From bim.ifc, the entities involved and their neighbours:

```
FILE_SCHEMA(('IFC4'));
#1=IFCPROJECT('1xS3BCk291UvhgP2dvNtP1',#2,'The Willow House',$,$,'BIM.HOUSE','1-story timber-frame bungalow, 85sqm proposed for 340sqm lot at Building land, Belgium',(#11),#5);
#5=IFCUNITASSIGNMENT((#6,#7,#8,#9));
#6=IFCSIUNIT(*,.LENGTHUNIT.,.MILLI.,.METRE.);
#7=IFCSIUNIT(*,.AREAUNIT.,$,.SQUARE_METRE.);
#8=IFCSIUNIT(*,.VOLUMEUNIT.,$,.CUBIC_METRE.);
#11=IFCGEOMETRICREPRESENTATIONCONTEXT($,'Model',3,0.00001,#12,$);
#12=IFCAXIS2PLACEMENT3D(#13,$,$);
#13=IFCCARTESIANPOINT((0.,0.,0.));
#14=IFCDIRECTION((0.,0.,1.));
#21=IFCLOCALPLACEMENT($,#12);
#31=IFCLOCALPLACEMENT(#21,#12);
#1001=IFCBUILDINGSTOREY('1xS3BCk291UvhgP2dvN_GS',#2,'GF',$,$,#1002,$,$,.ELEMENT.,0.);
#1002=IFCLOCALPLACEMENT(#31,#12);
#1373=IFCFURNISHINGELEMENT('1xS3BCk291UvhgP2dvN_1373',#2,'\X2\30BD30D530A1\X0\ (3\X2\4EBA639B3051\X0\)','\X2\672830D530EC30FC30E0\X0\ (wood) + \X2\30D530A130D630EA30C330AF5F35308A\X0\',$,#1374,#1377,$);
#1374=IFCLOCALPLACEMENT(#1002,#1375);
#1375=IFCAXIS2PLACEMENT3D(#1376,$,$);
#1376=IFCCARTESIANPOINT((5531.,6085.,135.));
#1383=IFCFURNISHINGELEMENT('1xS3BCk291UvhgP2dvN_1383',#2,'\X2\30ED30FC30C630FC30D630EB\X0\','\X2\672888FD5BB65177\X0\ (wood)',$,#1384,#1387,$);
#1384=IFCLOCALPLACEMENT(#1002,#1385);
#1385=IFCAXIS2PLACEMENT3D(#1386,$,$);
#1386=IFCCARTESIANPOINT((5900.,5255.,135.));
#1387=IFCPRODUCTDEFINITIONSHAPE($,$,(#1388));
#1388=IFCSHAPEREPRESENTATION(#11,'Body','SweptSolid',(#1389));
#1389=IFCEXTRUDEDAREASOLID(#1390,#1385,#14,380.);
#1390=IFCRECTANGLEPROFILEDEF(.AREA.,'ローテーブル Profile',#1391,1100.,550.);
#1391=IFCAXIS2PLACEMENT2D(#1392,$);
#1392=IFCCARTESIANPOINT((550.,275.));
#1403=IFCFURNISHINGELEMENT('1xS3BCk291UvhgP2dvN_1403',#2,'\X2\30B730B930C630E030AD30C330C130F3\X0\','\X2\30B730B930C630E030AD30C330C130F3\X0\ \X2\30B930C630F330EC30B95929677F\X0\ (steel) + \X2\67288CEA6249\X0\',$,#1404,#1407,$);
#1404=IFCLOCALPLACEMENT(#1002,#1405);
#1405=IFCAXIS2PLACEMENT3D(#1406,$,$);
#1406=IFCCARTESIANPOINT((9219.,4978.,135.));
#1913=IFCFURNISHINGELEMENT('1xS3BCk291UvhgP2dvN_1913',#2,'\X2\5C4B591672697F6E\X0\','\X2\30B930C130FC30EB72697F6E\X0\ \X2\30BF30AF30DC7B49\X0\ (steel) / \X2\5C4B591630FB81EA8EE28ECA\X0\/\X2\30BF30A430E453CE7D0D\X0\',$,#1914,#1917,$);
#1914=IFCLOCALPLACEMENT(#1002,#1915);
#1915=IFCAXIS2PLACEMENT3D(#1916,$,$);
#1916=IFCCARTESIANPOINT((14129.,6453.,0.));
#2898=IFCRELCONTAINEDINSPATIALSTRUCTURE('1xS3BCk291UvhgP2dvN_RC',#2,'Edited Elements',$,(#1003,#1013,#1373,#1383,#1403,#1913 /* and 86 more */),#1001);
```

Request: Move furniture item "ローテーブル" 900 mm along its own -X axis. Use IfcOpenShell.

```python
import ifcopenshell
import ifcopenshell.api.geometry
import ifcopenshell.util.placement

model = ifcopenshell.open("bim.ifc")

item = model.by_guid("1xS3BCk291UvhgP2dvN_1383")
matrix = ifcopenshell.util.placement.get_local_placement(item.ObjectPlacement)
matrix[:3, 3] -= matrix[:3, 0] * 900.0
ifcopenshell.api.geometry.edit_object_placement(model, product=item, matrix=matrix, is_si=False)

print(ifcopenshell.util.placement.get_local_placement(item.ObjectPlacement).round(3) + 0.0)

model.write("bim_v2.ifc")
```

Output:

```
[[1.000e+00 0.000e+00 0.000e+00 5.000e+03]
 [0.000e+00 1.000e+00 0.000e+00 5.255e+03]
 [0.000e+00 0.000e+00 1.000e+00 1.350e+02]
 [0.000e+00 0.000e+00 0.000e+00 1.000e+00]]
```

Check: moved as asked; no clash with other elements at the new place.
